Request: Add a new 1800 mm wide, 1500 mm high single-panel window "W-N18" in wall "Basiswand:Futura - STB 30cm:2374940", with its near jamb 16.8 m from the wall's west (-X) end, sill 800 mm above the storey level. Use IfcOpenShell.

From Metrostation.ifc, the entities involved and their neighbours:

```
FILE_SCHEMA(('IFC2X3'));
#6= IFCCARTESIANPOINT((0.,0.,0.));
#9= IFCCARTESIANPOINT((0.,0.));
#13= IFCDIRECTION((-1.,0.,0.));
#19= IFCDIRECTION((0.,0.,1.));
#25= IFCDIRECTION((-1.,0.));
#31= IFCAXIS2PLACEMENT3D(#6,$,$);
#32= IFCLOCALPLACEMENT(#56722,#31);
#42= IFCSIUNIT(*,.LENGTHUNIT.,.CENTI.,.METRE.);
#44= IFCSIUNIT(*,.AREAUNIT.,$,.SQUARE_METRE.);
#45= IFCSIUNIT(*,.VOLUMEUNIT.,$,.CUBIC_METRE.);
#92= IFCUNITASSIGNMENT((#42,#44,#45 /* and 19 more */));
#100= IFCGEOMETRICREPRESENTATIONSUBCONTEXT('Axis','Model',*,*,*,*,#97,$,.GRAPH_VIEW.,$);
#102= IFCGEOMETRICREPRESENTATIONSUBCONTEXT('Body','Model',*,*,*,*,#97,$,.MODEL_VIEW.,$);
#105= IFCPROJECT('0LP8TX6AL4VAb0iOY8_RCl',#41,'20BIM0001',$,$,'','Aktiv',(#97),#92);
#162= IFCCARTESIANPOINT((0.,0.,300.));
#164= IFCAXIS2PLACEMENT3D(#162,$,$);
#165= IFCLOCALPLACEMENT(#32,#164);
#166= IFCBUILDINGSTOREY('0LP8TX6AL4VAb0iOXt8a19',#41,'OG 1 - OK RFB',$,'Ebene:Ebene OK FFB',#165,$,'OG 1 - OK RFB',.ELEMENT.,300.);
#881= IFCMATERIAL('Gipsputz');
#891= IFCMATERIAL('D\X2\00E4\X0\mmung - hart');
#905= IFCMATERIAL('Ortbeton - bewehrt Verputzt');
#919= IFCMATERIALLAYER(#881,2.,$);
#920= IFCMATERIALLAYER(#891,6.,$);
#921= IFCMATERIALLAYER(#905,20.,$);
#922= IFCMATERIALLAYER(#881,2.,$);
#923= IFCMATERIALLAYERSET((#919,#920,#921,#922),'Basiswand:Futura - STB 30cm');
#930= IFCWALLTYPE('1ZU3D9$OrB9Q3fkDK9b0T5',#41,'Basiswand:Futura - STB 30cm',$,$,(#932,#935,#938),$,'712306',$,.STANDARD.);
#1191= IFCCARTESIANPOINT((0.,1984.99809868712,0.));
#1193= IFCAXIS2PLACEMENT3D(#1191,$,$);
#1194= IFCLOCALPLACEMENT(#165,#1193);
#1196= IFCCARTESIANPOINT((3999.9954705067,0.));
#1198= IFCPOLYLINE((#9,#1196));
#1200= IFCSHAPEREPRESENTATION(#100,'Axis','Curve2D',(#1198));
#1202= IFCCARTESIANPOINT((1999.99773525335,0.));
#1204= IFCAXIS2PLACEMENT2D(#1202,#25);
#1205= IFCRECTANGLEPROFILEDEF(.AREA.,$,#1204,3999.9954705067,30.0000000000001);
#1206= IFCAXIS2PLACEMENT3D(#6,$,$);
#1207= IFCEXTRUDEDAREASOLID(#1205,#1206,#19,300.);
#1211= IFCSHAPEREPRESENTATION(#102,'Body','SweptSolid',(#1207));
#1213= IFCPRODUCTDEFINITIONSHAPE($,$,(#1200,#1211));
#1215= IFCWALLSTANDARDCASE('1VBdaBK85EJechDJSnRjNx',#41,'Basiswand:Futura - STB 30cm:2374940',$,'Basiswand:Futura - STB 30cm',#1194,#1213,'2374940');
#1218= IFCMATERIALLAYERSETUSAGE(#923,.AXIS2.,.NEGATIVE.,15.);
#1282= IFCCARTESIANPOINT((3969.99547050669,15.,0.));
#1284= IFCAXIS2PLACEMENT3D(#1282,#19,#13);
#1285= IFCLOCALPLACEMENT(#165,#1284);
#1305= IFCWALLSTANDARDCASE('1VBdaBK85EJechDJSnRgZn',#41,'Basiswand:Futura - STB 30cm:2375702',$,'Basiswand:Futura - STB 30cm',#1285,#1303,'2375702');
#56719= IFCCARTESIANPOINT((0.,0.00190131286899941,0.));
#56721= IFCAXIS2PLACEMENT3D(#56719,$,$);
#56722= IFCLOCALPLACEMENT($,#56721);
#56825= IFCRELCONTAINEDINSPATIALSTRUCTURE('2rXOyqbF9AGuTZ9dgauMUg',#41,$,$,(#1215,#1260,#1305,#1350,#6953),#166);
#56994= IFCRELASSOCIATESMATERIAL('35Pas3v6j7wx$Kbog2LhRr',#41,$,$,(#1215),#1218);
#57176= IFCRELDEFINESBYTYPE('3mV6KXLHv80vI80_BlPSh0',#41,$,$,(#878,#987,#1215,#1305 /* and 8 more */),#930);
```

```python
import numpy as np
import ifcopenshell
import ifcopenshell.api.feature
import ifcopenshell.api.geometry
import ifcopenshell.api.root
import ifcopenshell.api.spatial
import ifcopenshell.api.type
import ifcopenshell.geom
import ifcopenshell.util.element
import ifcopenshell.util.placement
import ifcopenshell.util.representation
import ifcopenshell.util.shape
import ifcopenshell.util.unit

model = ifcopenshell.open("Metrostation.ifc")
unit_scale = ifcopenshell.util.unit.calculate_unit_scale(model)
settings = ifcopenshell.geom.settings()


def volume(element):
    """Net volume in cubic metres, openings subtracted."""
    shape = ifcopenshell.geom.create_shape(settings, element)
    return ifcopenshell.util.shape.get_volume(shape.geometry)


wall = model.by_guid("1VBdaBK85EJechDJSnRjNx")
storey = ifcopenshell.util.element.get_container(wall, ifc_class="IfcBuildingStorey")
context = ifcopenshell.util.representation.get_context(model, "Model", "Body", "MODEL_VIEW")
before = volume(wall)

width, height, from_end, sill = 1.8, 1.5, 16.8, 0.8  # metres

# The wall runs along its own X axis, and the end named is its -X end.
wall_shape = ifcopenshell.geom.create_shape(settings, wall)
x, y, z = ifcopenshell.util.shape.get_vertices(wall_shape.geometry).T
start = x.min() + from_end
face, thickness = float(y.min()), float(y.max() - y.min())
wall_matrix = ifcopenshell.util.placement.get_local_placement(wall.ObjectPlacement)
level = ifcopenshell.util.placement.get_local_placement(storey.ObjectPlacement)[2, 3]


def in_wall(x, y):
    """Placement at x, y metres in the wall's axes, at sill height."""
    matrix = wall_matrix.copy()
    matrix[:, 3] = wall_matrix @ np.array([x / unit_scale, y / unit_scale, 0.0, 1.0])
    matrix[2, 3] = level + sill / unit_scale
    return matrix


# Opening: a box that overshoots both wall faces by 50 mm.
opening = ifcopenshell.api.root.create_entity(model, ifc_class="IfcOpeningElement")
box = ifcopenshell.api.geometry.add_wall_representation(
    model, context=context, length=width, height=height, thickness=thickness + 0.1
)
ifcopenshell.api.geometry.assign_representation(model, product=opening, representation=box)
ifcopenshell.api.geometry.edit_object_placement(model, product=opening, matrix=in_wall(start, face - 0.05), is_si=False)
ifcopenshell.api.feature.add_feature(model, feature=opening, element=wall)

window = ifcopenshell.api.root.create_entity(model, ifc_class="IfcWindow", name="W-N18")
window.OverallWidth, window.OverallHeight = width / unit_scale, height / unit_scale
body = ifcopenshell.api.geometry.add_window_representation(
    model,
    context=context,
    overall_width=window.OverallWidth,
    overall_height=window.OverallHeight,
    partition_type="SINGLE_PANEL",
)
ifcopenshell.api.geometry.assign_representation(model, product=window, representation=body)
ifcopenshell.api.spatial.assign_container(model, products=[window], relating_structure=storey)
fills = ifcopenshell.api.feature.add_filling(model, opening=opening, element=window)
fills.OwnerHistory = window.OwnerHistory  # required in IFC2X3

# IFC2X3 keeps the operation on the window style.
style = ifcopenshell.api.root.create_entity(model, ifc_class="IfcWindowStyle", name="W-N18")
style.OperationType, style.ConstructionType = "SINGLE_PANEL", "NOTDEFINED"
style.ParameterTakesPrecedence = style.Sizeable = False
ifcopenshell.api.type.assign_type(model, related_objects=[window], relating_type=style)

# Centre the window in the wall's thickness.
ifcopenshell.api.geometry.edit_object_placement(model, product=window, matrix=in_wall(start, face), is_si=False)
window_shape = ifcopenshell.geom.create_shape(settings, window)
depth = ifcopenshell.util.shape.get_vertices(window_shape.geometry)[:, 1]
offset = face + thickness / 2 - (depth.min() + depth.max()) / 2
ifcopenshell.api.geometry.edit_object_placement(model, product=window, matrix=in_wall(start, offset), is_si=False)

after = volume(wall)

print(f"wall volume {before:.3f} -> {after:.3f} m3")

model.write("Metrostation_updated.ifc")
```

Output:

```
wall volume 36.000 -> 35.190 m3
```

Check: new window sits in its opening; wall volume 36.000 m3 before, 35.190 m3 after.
